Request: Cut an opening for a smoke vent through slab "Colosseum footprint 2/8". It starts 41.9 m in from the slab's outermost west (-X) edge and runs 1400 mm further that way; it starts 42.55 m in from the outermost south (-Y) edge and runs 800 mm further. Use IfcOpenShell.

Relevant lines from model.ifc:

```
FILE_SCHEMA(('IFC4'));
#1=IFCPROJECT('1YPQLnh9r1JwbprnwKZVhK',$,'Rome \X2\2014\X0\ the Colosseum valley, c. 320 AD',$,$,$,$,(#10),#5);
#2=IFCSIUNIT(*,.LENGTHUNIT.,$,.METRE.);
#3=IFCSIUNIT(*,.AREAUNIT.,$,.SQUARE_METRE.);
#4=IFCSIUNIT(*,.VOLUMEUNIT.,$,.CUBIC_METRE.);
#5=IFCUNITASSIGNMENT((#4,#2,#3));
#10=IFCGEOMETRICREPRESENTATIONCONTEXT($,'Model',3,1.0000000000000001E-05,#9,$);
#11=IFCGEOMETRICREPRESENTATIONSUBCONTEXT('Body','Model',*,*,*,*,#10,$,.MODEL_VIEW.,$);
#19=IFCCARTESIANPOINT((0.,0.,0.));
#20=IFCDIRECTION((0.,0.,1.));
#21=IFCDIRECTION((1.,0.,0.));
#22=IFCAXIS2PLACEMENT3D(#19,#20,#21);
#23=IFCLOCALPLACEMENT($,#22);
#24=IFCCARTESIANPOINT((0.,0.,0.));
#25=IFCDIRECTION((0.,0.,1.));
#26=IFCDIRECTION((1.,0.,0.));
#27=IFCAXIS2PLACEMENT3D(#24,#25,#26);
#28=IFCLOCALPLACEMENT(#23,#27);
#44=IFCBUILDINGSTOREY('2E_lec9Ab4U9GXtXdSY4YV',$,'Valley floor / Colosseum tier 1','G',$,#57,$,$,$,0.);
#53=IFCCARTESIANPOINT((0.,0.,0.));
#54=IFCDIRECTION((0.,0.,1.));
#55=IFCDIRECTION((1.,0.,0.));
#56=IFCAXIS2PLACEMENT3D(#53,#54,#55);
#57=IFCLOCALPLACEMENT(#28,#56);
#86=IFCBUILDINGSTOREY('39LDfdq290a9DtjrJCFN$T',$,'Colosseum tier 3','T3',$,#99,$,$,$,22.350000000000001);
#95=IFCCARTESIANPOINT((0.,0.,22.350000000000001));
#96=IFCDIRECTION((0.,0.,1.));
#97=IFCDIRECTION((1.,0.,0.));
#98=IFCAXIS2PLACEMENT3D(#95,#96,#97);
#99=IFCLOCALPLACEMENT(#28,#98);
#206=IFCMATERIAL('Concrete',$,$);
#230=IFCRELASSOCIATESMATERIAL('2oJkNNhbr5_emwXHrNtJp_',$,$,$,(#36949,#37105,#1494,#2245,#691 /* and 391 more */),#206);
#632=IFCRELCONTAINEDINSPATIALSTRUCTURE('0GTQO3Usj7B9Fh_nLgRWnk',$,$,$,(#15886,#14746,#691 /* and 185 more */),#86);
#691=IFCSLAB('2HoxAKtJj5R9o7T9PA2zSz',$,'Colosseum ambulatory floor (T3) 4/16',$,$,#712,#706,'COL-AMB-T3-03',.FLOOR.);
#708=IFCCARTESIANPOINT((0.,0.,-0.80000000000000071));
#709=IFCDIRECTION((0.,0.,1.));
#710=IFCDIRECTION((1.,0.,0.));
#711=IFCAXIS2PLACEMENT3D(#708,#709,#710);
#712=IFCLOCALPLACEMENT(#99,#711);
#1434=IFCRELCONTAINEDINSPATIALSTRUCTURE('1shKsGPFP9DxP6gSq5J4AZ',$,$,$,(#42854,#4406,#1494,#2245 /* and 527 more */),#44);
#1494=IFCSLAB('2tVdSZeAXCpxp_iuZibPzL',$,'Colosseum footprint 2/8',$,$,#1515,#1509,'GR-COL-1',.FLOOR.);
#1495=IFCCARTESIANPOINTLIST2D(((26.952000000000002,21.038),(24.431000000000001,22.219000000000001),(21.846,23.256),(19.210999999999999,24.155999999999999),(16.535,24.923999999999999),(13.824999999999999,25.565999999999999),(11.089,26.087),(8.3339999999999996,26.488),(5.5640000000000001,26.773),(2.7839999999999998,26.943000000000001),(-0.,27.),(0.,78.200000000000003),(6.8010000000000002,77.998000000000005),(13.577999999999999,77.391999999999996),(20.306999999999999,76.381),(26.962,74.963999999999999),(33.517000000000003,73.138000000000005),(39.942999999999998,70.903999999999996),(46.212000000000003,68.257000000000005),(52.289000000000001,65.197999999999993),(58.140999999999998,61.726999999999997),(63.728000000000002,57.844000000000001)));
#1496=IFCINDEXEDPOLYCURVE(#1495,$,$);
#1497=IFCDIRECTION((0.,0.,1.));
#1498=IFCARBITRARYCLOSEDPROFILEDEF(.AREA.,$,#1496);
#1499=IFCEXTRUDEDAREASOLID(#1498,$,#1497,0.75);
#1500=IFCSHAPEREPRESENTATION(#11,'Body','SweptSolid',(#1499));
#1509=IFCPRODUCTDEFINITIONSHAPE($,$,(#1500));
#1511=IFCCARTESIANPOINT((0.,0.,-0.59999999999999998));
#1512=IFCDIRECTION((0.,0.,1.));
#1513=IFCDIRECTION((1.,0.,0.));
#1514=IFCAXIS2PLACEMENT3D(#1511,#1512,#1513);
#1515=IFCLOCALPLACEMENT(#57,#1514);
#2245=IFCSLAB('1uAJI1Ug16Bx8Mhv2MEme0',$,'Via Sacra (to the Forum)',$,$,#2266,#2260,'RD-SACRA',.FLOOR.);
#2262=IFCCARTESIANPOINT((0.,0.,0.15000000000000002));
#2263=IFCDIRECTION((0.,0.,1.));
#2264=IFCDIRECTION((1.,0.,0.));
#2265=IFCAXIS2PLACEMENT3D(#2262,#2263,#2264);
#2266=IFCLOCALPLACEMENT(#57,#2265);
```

```python
import numpy as np
import ifcopenshell
import ifcopenshell.api.feature
import ifcopenshell.api.geometry
import ifcopenshell.api.root
import ifcopenshell.geom
import ifcopenshell.util.placement
import ifcopenshell.util.representation
import ifcopenshell.util.shape
import ifcopenshell.util.unit

model = ifcopenshell.open("model.ifc")
unit_scale = ifcopenshell.util.unit.calculate_unit_scale(model)
settings = ifcopenshell.geom.settings()


def volume(element):
    """Net volume in cubic metres, openings subtracted."""
    shape = ifcopenshell.geom.create_shape(settings, element)
    return ifcopenshell.util.shape.get_volume(shape.geometry)


slab = model.by_id(1494)
before = volume(slab)

# Extent in the slab's own axes, in metres. The edges named are its -X and -Y sides.
slab_shape = ifcopenshell.geom.create_shape(settings, slab)
vertices = ifcopenshell.util.shape.get_vertices(slab_shape.geometry)
x_min, y_min, bottom = vertices.min(axis=0)
top = vertices[:, 2].max()

opening = ifcopenshell.api.root.create_entity(model, ifc_class="IfcOpeningElement", name="Smoke vent opening", predefined_type="OPENING")
context = ifcopenshell.util.representation.get_context(model, "Model", "Body", "MODEL_VIEW")
width, depth = 1.4, 0.8
outline = [(0.0, 0.0), (width, 0.0), (width, depth), (0.0, depth), (0.0, 0.0)]
# Overshoot both faces by 50 mm so the cut is clean.
shape = ifcopenshell.api.geometry.add_slab_representation(
    model, context=context, depth=top - bottom + 0.1, polyline=outline
)
ifcopenshell.api.geometry.assign_representation(model, product=opening, representation=shape)

matrix = ifcopenshell.util.placement.get_local_placement(slab.ObjectPlacement)
matrix[:, 3] = matrix @ np.append(np.array([x_min + 41.9, y_min + 42.55, bottom - 0.05]) / unit_scale, 1.0)
ifcopenshell.api.geometry.edit_object_placement(model, product=opening, matrix=matrix, is_si=False)
ifcopenshell.api.feature.add_feature(model, feature=opening, element=slab)

after = volume(slab)

print(f"slab volume {before:.3f} -> {after:.3f} m3")

model.write("model_edited.ifc")
```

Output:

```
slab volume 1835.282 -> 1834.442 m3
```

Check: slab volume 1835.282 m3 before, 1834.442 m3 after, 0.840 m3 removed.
